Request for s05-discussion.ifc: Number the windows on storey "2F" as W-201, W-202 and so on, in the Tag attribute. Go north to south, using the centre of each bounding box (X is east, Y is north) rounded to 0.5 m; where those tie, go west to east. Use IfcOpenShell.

First a look at what the model holds.

```python
import ifcopenshell
import ifcopenshell.util.element
import ifcopenshell.util.placement

model = ifcopenshell.open("s05-discussion.ifc")
print(model.schema)
storey = next(s for s in model.by_type("IfcBuildingStorey") if s.Name == "2F")
windows = [e for e in ifcopenshell.util.element.get_decomposition(storey) if e.is_a("IfcWindow")]
for e in sorted(windows, key=lambda e: e.id()):
    origin = ifcopenshell.util.placement.get_local_placement(e.ObjectPlacement)[:3, 3]
    print(e.id(), e.Tag, e.Name, origin.round(2) + 0.0, sep=" | ")
```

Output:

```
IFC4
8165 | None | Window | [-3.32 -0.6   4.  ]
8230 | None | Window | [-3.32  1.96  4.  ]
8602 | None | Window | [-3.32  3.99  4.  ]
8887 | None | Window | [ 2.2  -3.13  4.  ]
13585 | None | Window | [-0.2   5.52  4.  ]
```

```python
import ifcopenshell
import ifcopenshell.geom
import ifcopenshell.util.element
import ifcopenshell.util.shape

model = ifcopenshell.open("s05-discussion.ifc")
settings = ifcopenshell.geom.settings()
settings.set("use-world-coords", True)


def centre(element):
    shape = ifcopenshell.geom.create_shape(settings, element)
    return ifcopenshell.util.shape.get_bbox_centroid(shape.geometry)


storey = next(s for s in model.by_type("IfcBuildingStorey") if s.Name == "2F")
windows = [e for e in ifcopenshell.util.element.get_decomposition(storey) if e.is_a("IfcWindow")]

# Insertion points can sit at a corner or the storey origin, so sort by the geometry (in metres).
centres = {e: centre(e) for e in windows}
windows.sort(key=lambda e: (-round(centres[e][1] / 0.5), centres[e][0]))

for i, e in enumerate(windows, start=1):
    number = f"W-2{i:02d}"
    e.Tag = number
    print(e.id(), number)

model.write("s05-discussion_rev.ifc")
```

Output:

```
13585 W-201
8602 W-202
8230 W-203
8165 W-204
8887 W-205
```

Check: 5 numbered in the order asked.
